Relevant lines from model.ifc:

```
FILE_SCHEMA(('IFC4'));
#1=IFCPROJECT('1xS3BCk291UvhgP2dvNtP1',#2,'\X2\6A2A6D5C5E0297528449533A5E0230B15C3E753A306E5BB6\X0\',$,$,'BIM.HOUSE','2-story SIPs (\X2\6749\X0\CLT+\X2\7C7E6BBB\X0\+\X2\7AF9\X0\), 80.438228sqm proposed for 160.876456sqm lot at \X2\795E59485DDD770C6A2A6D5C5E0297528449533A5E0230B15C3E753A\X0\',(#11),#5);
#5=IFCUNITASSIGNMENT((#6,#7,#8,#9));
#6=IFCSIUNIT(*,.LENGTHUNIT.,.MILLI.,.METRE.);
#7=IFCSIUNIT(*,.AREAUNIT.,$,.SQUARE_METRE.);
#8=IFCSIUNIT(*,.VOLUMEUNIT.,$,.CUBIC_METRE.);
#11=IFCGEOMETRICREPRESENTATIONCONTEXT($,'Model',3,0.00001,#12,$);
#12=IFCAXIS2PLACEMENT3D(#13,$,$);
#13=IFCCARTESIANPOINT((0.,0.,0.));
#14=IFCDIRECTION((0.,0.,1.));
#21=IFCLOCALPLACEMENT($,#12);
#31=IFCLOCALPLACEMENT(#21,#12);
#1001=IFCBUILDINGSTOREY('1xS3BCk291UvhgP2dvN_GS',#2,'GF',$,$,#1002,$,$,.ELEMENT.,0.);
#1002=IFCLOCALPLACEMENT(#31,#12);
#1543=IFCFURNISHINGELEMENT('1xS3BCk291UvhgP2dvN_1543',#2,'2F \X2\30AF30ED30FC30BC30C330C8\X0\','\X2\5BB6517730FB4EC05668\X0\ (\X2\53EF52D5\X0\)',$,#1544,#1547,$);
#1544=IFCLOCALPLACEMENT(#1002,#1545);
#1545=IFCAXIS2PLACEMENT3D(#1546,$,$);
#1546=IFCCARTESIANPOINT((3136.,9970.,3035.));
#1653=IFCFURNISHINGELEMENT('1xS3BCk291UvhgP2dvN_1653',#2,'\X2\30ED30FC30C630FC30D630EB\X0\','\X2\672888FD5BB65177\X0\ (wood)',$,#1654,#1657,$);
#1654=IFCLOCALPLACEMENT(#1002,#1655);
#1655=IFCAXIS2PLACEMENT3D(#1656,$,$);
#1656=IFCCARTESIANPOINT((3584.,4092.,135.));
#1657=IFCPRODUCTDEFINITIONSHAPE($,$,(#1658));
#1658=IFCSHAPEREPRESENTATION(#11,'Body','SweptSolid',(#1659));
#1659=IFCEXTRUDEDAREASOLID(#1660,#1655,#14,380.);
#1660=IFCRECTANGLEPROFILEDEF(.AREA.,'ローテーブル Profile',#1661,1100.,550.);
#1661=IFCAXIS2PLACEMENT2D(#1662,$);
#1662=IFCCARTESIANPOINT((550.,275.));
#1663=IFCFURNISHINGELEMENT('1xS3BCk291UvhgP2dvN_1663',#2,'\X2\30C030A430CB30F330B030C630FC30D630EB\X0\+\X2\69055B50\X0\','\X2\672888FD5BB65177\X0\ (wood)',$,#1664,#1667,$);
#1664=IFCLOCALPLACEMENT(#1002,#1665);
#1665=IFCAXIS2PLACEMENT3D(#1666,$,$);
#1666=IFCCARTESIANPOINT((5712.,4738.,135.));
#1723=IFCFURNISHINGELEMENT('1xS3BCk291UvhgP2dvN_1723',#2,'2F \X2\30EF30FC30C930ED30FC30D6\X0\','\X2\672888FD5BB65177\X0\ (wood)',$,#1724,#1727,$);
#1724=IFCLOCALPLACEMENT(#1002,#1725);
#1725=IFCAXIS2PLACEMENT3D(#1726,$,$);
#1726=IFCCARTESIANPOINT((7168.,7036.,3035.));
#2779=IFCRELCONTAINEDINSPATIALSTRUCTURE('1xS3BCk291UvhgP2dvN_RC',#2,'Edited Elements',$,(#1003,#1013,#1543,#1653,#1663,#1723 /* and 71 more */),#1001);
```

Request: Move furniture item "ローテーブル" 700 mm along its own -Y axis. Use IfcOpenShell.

```python
import ifcopenshell
import ifcopenshell.api.geometry
import ifcopenshell.util.placement

model = ifcopenshell.open("model.ifc")

item = model.by_guid("1xS3BCk291UvhgP2dvN_1653")
matrix = ifcopenshell.util.placement.get_local_placement(item.ObjectPlacement)
matrix[:3, 3] -= matrix[:3, 1] * 700.0
ifcopenshell.api.geometry.edit_object_placement(model, product=item, matrix=matrix, is_si=False)

print(ifcopenshell.util.placement.get_local_placement(item.ObjectPlacement).round(3) + 0.0)

model.write("model-out.ifc")
```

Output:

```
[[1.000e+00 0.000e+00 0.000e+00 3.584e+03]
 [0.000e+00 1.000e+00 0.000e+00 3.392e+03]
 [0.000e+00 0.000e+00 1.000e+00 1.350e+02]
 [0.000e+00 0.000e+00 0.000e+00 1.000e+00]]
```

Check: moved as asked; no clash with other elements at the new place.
